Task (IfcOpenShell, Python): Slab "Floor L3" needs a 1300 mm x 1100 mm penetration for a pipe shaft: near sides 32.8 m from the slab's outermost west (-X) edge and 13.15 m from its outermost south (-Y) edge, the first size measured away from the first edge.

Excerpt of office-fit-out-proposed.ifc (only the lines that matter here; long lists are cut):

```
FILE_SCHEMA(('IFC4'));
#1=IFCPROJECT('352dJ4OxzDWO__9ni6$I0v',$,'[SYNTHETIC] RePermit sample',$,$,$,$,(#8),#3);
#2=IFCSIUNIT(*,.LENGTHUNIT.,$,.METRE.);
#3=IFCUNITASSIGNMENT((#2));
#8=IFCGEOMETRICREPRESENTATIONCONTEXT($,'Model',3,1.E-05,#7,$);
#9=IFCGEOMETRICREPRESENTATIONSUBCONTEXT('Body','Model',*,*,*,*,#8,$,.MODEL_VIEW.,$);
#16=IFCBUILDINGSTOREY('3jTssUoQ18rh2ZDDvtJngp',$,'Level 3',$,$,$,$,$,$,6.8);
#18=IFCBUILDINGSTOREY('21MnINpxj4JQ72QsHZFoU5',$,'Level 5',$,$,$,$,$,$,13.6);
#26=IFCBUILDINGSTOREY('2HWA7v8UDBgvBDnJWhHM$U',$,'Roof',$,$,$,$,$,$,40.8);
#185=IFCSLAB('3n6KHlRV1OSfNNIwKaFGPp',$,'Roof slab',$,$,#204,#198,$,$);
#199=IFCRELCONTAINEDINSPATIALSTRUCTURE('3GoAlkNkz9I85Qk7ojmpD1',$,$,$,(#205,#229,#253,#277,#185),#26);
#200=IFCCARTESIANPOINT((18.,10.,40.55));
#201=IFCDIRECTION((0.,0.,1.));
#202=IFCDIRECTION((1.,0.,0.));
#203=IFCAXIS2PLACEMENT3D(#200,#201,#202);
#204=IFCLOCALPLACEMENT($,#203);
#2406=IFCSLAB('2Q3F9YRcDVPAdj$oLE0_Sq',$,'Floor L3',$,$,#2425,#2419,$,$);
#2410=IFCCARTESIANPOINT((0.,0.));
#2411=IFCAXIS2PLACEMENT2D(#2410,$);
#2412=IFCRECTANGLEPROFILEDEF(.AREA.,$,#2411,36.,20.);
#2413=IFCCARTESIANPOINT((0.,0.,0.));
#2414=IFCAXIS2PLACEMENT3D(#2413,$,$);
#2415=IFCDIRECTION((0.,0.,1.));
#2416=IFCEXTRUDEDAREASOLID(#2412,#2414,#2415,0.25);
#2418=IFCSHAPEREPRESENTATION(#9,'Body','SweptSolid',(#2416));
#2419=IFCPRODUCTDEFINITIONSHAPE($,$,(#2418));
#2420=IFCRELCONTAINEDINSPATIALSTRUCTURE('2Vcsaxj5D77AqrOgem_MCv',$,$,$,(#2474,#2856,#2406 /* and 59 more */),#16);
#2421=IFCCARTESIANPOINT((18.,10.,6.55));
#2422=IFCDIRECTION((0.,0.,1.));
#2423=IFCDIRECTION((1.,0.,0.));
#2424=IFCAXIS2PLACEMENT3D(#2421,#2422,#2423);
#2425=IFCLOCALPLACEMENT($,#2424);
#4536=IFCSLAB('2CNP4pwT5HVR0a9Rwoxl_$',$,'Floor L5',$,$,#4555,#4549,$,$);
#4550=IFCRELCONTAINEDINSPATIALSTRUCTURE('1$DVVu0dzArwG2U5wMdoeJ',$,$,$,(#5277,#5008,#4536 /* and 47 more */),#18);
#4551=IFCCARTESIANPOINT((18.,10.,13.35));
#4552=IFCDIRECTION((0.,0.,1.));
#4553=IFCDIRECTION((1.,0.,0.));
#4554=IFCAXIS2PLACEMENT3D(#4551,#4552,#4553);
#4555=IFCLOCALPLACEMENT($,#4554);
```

```python
import numpy as np
import ifcopenshell
import ifcopenshell.api.feature
import ifcopenshell.api.geometry
import ifcopenshell.api.root
import ifcopenshell.geom
import ifcopenshell.util.placement
import ifcopenshell.util.representation
import ifcopenshell.util.shape
import ifcopenshell.util.unit

model = ifcopenshell.open("office-fit-out-proposed.ifc")
unit_scale = ifcopenshell.util.unit.calculate_unit_scale(model)
settings = ifcopenshell.geom.settings()


def volume(element):
    """Net volume in cubic metres, openings subtracted."""
    shape = ifcopenshell.geom.create_shape(settings, element)
    return ifcopenshell.util.shape.get_volume(shape.geometry)


slab = model.by_guid("2Q3F9YRcDVPAdj$oLE0_Sq")
before = volume(slab)

# Extent in the slab's own axes, in metres. The edges named are its -X and -Y sides.
slab_shape = ifcopenshell.geom.create_shape(settings, slab)
vertices = ifcopenshell.util.shape.get_vertices(slab_shape.geometry)
x_min, y_min, bottom = vertices.min(axis=0)
top = vertices[:, 2].max()

opening = ifcopenshell.api.root.create_entity(model, ifc_class="IfcOpeningElement", name="Pipe shaft opening", predefined_type="OPENING")
context = ifcopenshell.util.representation.get_context(model, "Model", "Body", "MODEL_VIEW")
width, depth = 1.3, 1.1
outline = [(0.0, 0.0), (width, 0.0), (width, depth), (0.0, depth), (0.0, 0.0)]
# Overshoot both faces by 50 mm so the cut is clean.
shape = ifcopenshell.api.geometry.add_slab_representation(
    model, context=context, depth=top - bottom + 0.1, polyline=outline
)
ifcopenshell.api.geometry.assign_representation(model, product=opening, representation=shape)

matrix = ifcopenshell.util.placement.get_local_placement(slab.ObjectPlacement)
matrix[:, 3] = matrix @ np.append(np.array([x_min + 32.8, y_min + 13.15, bottom - 0.05]) / unit_scale, 1.0)
ifcopenshell.api.geometry.edit_object_placement(model, product=opening, matrix=matrix, is_si=False)
ifcopenshell.api.feature.add_feature(model, feature=opening, element=slab)

after = volume(slab)

print(f"slab volume {before:.3f} -> {after:.3f} m3")

model.write("office-fit-out-proposed_updated.ifc")
```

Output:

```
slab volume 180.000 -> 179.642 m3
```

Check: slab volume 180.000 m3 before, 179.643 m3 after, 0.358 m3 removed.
